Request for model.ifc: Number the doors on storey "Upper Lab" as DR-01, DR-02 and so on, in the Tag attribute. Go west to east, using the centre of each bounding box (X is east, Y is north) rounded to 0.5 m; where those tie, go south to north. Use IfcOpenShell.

First a look at what the model holds.

```python
import ifcopenshell
import ifcopenshell.util.element
import ifcopenshell.util.placement

model = ifcopenshell.open("model.ifc")
print(model.schema)
storey = next(s for s in model.by_type("IfcBuildingStorey") if s.Name == "Upper Lab")
doors = [e for e in ifcopenshell.util.element.get_decomposition(storey) if e.is_a("IfcDoor")]
for e in sorted(doors, key=lambda e: e.id()):
    origin = ifcopenshell.util.placement.get_local_placement(e.ObjectPlacement)[:3, 3]
    print(e.id(), e.Tag, e.Name, origin.round(2) + 0.0, sep=" | ")
```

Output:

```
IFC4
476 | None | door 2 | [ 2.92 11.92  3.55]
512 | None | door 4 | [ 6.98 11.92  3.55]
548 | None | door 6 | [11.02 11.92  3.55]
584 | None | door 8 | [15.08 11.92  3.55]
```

```python
import ifcopenshell
import ifcopenshell.geom
import ifcopenshell.util.element
import ifcopenshell.util.shape

model = ifcopenshell.open("model.ifc")
settings = ifcopenshell.geom.settings()
settings.set("use-world-coords", True)


def centre(element):
    shape = ifcopenshell.geom.create_shape(settings, element)
    return ifcopenshell.util.shape.get_bbox_centroid(shape.geometry)


storey = next(s for s in model.by_type("IfcBuildingStorey") if s.Name == "Upper Lab")
doors = [e for e in ifcopenshell.util.element.get_decomposition(storey) if e.is_a("IfcDoor")]

# Insertion points can sit at a corner or the storey origin, so sort by the geometry (in metres).
centres = {e: centre(e) for e in doors}
doors.sort(key=lambda e: (round(centres[e][0] / 0.5), centres[e][1]))

for i, e in enumerate(doors, start=1):
    number = f"DR-{i:02d}"
    e.Tag = number
    print(e.id(), number)

model.write("model_rev.ifc")
```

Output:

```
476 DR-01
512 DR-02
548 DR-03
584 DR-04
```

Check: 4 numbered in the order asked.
